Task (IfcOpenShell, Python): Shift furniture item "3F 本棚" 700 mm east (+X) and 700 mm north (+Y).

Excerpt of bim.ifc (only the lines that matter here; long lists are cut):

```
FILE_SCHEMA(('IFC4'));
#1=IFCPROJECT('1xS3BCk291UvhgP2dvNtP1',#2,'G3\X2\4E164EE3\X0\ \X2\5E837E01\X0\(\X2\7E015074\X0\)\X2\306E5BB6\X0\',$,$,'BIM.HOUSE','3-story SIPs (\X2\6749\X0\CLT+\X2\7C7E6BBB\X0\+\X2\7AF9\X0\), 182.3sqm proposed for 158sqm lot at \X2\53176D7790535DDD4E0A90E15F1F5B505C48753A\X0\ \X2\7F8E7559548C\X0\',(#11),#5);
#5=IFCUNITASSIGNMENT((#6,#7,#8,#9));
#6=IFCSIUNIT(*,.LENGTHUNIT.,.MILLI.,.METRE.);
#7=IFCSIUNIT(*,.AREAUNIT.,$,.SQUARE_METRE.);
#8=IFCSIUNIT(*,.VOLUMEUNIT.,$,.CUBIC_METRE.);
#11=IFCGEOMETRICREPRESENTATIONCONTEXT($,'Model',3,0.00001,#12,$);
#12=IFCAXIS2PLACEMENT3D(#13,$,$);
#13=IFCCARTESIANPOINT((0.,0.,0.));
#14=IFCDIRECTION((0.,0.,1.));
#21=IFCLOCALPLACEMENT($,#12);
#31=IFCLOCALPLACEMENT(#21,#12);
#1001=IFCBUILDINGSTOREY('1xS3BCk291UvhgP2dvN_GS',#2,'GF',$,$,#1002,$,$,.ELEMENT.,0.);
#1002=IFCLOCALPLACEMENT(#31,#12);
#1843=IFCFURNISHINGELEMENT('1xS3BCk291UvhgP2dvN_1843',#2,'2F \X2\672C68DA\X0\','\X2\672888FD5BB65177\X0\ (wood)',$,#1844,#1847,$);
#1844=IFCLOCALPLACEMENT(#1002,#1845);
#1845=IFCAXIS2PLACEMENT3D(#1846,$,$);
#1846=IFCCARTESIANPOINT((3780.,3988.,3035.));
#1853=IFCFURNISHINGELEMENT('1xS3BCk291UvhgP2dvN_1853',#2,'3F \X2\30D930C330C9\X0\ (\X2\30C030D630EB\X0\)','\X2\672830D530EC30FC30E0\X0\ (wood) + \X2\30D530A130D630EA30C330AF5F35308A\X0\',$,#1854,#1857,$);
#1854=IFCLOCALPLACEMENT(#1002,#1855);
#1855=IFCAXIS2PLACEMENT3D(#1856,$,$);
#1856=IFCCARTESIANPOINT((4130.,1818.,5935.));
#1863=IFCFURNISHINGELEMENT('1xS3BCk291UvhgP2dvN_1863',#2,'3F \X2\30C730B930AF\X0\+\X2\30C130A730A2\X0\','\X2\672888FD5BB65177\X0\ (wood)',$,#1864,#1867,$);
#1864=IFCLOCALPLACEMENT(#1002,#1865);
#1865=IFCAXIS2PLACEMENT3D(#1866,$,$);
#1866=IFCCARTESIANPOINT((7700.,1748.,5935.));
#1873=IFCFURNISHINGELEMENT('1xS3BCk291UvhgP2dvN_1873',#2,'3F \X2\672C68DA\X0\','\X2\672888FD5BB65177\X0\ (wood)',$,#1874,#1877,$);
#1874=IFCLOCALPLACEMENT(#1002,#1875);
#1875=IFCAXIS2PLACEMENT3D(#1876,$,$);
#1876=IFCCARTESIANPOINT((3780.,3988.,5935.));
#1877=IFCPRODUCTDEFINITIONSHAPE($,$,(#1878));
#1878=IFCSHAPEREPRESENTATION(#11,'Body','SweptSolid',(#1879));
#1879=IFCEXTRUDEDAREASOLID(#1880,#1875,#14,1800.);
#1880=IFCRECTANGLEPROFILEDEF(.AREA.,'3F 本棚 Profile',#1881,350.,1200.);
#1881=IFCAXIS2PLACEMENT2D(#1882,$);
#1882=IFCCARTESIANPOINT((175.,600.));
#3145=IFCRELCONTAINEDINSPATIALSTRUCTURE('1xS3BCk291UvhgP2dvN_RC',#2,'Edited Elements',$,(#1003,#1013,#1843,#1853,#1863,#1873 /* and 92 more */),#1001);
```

```python
import ifcopenshell
import ifcopenshell.api.geometry
import ifcopenshell.util.placement

model = ifcopenshell.open("bim.ifc")

item = model.by_guid("1xS3BCk291UvhgP2dvN_1873")
matrix = ifcopenshell.util.placement.get_local_placement(item.ObjectPlacement)
matrix[0, 3] += 700.0
matrix[1, 3] += 700.0
ifcopenshell.api.geometry.edit_object_placement(model, product=item, matrix=matrix, is_si=False)

print(ifcopenshell.util.placement.get_local_placement(item.ObjectPlacement).round(3) + 0.0)

model.write("bim_rev.ifc")
```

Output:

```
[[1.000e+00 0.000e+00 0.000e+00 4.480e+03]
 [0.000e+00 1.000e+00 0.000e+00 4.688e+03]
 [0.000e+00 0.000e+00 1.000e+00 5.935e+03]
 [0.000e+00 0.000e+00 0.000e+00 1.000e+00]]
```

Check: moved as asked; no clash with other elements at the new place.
